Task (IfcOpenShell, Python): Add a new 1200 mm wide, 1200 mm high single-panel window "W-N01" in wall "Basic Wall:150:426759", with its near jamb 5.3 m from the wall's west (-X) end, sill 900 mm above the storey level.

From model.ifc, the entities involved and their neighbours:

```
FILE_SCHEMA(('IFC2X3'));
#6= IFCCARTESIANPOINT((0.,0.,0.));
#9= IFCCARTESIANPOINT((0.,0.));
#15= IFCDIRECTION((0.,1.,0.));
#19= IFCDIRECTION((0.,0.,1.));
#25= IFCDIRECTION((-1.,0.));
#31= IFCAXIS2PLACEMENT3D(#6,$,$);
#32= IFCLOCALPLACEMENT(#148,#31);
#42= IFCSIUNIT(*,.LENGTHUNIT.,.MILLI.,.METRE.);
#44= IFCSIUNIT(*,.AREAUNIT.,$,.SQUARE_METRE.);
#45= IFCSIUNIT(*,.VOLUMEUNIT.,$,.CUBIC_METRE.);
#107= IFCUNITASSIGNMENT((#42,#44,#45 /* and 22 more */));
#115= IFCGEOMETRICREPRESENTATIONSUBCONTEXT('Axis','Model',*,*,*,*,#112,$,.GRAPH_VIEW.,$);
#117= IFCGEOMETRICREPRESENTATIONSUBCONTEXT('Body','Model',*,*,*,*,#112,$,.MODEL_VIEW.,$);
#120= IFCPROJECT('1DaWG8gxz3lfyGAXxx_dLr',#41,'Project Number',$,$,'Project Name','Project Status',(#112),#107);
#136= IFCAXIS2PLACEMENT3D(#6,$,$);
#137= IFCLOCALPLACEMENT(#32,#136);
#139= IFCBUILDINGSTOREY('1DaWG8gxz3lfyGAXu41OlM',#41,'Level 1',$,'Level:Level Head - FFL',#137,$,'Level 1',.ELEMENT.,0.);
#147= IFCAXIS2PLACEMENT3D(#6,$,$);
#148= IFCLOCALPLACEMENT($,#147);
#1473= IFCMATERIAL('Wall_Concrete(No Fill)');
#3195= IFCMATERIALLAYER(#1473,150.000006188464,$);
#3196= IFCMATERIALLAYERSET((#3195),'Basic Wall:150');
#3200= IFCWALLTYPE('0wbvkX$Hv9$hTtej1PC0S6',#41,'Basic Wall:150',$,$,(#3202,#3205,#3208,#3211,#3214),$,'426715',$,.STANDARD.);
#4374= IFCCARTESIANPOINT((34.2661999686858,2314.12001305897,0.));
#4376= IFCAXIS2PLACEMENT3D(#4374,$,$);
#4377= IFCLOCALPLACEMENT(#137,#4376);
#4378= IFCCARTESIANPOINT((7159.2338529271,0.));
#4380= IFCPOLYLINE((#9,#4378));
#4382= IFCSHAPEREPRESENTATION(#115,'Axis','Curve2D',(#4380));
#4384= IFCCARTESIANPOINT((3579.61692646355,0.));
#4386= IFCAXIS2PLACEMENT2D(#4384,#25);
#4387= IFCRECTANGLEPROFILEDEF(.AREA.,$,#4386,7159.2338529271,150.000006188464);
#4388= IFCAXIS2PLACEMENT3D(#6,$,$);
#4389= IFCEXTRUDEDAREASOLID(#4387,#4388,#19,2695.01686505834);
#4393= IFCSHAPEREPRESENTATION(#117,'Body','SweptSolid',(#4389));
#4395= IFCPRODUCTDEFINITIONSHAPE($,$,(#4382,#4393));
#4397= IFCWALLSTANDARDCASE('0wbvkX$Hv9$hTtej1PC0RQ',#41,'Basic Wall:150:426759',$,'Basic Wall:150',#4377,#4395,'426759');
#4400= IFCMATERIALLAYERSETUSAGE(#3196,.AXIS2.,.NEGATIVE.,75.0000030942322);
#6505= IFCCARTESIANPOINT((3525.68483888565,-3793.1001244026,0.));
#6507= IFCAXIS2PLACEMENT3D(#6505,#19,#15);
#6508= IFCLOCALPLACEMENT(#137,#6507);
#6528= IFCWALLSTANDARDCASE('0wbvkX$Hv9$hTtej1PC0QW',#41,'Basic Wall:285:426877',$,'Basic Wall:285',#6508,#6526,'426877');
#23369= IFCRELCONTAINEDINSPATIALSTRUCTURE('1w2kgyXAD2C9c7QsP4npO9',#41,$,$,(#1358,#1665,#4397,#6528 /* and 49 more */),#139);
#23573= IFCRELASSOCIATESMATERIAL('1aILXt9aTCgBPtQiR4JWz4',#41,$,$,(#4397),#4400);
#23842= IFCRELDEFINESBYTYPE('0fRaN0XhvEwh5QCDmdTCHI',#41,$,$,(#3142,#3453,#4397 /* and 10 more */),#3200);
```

```python
import numpy as np
import ifcopenshell
import ifcopenshell.api.feature
import ifcopenshell.api.geometry
import ifcopenshell.api.root
import ifcopenshell.api.spatial
import ifcopenshell.api.type
import ifcopenshell.geom
import ifcopenshell.util.element
import ifcopenshell.util.placement
import ifcopenshell.util.representation
import ifcopenshell.util.shape
import ifcopenshell.util.unit

model = ifcopenshell.open("model.ifc")
unit_scale = ifcopenshell.util.unit.calculate_unit_scale(model)
settings = ifcopenshell.geom.settings()


def volume(element):
    """Net volume in cubic metres, openings subtracted."""
    shape = ifcopenshell.geom.create_shape(settings, element)
    return ifcopenshell.util.shape.get_volume(shape.geometry)


wall = model.by_guid("0wbvkX$Hv9$hTtej1PC0RQ")
storey = ifcopenshell.util.element.get_container(wall, ifc_class="IfcBuildingStorey")
context = ifcopenshell.util.representation.get_context(model, "Model", "Body", "MODEL_VIEW")
before = volume(wall)

width, height, from_end, sill = 1.2, 1.2, 5.3, 0.9  # metres

# The wall runs along its own X axis, and the end named is its -X end.
wall_shape = ifcopenshell.geom.create_shape(settings, wall)
x, y, z = ifcopenshell.util.shape.get_vertices(wall_shape.geometry).T
start = x.min() + from_end
face, thickness = float(y.min()), float(y.max() - y.min())
wall_matrix = ifcopenshell.util.placement.get_local_placement(wall.ObjectPlacement)
level = ifcopenshell.util.placement.get_local_placement(storey.ObjectPlacement)[2, 3]


def in_wall(x, y):
    """Placement at x, y metres in the wall's axes, at sill height."""
    matrix = wall_matrix.copy()
    matrix[:, 3] = wall_matrix @ np.array([x / unit_scale, y / unit_scale, 0.0, 1.0])
    matrix[2, 3] = level + sill / unit_scale
    return matrix


# Opening: a box that overshoots both wall faces by 50 mm.
opening = ifcopenshell.api.root.create_entity(model, ifc_class="IfcOpeningElement")
box = ifcopenshell.api.geometry.add_wall_representation(
    model, context=context, length=width, height=height, thickness=thickness + 0.1
)
ifcopenshell.api.geometry.assign_representation(model, product=opening, representation=box)
ifcopenshell.api.geometry.edit_object_placement(model, product=opening, matrix=in_wall(start, face - 0.05), is_si=False)
ifcopenshell.api.feature.add_feature(model, feature=opening, element=wall)

window = ifcopenshell.api.root.create_entity(model, ifc_class="IfcWindow", name="W-N01")
window.OverallWidth, window.OverallHeight = width / unit_scale, height / unit_scale
body = ifcopenshell.api.geometry.add_window_representation(
    model,
    context=context,
    overall_width=window.OverallWidth,
    overall_height=window.OverallHeight,
    partition_type="SINGLE_PANEL",
)
ifcopenshell.api.geometry.assign_representation(model, product=window, representation=body)
ifcopenshell.api.spatial.assign_container(model, products=[window], relating_structure=storey)
fills = ifcopenshell.api.feature.add_filling(model, opening=opening, element=window)
fills.OwnerHistory = window.OwnerHistory  # required in IFC2X3

# IFC2X3 keeps the operation on the window style.
style = ifcopenshell.api.root.create_entity(model, ifc_class="IfcWindowStyle", name="W-N01")
style.OperationType, style.ConstructionType = "SINGLE_PANEL", "NOTDEFINED"
style.ParameterTakesPrecedence = style.Sizeable = False
ifcopenshell.api.type.assign_type(model, related_objects=[window], relating_type=style)

# Centre the window in the wall's thickness.
ifcopenshell.api.geometry.edit_object_placement(model, product=window, matrix=in_wall(start, face), is_si=False)
window_shape = ifcopenshell.geom.create_shape(settings, window)
depth = ifcopenshell.util.shape.get_vertices(window_shape.geometry)[:, 1]
offset = face + thickness / 2 - (depth.min() + depth.max()) / 2
ifcopenshell.api.geometry.edit_object_placement(model, product=window, matrix=in_wall(start, offset), is_si=False)

after = volume(wall)

print(f"wall volume {before:.3f} -> {after:.3f} m3")

model.write("model_v2.ifc")
```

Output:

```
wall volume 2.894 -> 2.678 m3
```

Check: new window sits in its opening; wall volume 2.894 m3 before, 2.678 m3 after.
